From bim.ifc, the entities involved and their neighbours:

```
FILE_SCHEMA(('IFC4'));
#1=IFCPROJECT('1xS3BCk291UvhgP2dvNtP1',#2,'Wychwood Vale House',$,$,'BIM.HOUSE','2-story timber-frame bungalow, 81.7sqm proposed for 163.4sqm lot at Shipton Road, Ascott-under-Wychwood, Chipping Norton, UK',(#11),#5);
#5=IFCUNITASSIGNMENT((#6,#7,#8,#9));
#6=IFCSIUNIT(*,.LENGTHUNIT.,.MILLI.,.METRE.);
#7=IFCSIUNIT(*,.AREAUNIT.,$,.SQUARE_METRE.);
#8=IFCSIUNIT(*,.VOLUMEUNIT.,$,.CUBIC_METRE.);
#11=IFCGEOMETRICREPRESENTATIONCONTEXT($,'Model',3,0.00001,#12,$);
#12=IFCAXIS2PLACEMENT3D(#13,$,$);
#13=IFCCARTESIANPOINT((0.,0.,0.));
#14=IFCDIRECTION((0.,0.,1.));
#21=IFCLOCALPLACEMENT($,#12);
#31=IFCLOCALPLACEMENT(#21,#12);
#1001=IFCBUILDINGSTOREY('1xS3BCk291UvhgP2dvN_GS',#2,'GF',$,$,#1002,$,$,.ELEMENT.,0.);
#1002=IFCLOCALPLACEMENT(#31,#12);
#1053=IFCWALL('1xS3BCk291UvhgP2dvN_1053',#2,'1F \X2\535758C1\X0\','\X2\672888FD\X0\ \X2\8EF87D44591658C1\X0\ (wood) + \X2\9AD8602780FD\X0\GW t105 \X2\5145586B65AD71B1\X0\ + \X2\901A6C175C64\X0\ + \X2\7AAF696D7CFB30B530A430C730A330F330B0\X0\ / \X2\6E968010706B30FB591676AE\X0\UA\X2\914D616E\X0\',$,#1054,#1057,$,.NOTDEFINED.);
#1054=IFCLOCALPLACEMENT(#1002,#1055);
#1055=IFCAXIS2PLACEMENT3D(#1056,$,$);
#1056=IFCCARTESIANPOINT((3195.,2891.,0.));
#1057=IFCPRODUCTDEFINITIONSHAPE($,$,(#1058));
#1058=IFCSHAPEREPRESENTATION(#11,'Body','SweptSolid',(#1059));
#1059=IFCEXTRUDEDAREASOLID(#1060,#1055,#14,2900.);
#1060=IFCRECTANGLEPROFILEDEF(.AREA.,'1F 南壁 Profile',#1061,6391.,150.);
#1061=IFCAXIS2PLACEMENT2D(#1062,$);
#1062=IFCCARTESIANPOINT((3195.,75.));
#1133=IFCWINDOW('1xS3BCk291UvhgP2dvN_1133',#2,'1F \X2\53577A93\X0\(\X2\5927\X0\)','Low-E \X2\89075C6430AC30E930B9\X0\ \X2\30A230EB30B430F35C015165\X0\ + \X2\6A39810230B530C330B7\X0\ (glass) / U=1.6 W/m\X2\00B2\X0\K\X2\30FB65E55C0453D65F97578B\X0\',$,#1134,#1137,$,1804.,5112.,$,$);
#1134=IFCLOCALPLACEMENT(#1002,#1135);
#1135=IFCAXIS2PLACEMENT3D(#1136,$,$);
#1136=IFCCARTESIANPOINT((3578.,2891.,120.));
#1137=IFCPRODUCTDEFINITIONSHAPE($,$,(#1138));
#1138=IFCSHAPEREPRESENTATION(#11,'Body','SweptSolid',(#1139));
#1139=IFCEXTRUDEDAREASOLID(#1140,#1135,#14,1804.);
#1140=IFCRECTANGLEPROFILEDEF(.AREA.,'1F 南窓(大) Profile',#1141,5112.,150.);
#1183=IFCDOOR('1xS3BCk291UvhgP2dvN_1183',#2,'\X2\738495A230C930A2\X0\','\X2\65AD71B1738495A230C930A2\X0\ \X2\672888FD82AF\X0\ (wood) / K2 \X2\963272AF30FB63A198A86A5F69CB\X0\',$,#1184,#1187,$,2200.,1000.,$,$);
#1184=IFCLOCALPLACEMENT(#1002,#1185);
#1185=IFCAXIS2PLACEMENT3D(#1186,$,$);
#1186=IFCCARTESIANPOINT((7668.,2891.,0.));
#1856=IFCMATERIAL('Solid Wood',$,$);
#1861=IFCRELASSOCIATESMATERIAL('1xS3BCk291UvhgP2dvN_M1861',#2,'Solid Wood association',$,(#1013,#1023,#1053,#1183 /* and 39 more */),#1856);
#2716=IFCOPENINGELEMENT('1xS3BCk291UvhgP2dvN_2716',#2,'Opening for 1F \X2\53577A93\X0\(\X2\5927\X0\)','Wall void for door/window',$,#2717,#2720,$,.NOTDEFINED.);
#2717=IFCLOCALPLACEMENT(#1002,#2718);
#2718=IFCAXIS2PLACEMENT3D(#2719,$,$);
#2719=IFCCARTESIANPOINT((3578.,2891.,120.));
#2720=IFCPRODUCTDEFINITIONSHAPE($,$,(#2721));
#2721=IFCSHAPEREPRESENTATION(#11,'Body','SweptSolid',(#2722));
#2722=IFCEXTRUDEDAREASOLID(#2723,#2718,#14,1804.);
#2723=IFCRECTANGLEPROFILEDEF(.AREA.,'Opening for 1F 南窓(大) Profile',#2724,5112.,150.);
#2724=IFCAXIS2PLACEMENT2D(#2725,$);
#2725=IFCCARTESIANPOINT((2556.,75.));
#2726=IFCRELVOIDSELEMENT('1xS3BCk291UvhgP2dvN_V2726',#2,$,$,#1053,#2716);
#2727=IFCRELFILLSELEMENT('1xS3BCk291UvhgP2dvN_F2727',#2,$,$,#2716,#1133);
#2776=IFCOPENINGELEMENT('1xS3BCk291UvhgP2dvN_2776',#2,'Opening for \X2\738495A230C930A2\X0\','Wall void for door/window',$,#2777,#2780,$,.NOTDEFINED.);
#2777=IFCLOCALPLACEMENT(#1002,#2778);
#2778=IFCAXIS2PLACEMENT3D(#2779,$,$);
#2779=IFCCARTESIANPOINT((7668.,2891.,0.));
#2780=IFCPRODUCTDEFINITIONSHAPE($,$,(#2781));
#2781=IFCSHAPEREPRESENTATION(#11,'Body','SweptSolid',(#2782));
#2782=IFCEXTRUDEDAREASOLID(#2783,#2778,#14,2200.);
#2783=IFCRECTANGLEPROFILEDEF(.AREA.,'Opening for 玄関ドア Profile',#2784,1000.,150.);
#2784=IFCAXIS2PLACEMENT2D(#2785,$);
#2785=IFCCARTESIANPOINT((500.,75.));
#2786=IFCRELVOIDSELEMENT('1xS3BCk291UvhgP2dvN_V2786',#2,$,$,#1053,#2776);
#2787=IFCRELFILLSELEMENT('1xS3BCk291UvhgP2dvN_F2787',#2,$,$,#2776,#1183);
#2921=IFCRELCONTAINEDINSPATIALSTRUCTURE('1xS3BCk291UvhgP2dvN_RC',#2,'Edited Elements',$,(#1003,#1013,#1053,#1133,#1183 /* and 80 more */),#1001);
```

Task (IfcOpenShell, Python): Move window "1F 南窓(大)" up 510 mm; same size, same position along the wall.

```python
import numpy as np
import ifcopenshell
import ifcopenshell.api.geometry
import ifcopenshell.util.placement
import ifcopenshell.util.unit

model = ifcopenshell.open("bim.ifc")
unit_scale = ifcopenshell.util.unit.calculate_unit_scale(model)

window = model.by_id(1133)
opening = window.FillsVoids[0].RelatingOpeningElement
dz = 0.51 / unit_scale

shift = np.array([0.0, 0.0, dz])
# The window is not placed relative to its opening, so move both.
for product in (opening, window):
    matrix = ifcopenshell.util.placement.get_local_placement(product.ObjectPlacement)
    matrix[:3, 3] += shift
    ifcopenshell.api.geometry.edit_object_placement(model, product=product, matrix=matrix, is_si=False)

print(f"moved by {dz * unit_scale:+.3f} m")

model.write("bim-out.ifc")
```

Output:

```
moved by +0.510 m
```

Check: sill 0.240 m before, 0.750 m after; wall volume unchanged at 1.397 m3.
